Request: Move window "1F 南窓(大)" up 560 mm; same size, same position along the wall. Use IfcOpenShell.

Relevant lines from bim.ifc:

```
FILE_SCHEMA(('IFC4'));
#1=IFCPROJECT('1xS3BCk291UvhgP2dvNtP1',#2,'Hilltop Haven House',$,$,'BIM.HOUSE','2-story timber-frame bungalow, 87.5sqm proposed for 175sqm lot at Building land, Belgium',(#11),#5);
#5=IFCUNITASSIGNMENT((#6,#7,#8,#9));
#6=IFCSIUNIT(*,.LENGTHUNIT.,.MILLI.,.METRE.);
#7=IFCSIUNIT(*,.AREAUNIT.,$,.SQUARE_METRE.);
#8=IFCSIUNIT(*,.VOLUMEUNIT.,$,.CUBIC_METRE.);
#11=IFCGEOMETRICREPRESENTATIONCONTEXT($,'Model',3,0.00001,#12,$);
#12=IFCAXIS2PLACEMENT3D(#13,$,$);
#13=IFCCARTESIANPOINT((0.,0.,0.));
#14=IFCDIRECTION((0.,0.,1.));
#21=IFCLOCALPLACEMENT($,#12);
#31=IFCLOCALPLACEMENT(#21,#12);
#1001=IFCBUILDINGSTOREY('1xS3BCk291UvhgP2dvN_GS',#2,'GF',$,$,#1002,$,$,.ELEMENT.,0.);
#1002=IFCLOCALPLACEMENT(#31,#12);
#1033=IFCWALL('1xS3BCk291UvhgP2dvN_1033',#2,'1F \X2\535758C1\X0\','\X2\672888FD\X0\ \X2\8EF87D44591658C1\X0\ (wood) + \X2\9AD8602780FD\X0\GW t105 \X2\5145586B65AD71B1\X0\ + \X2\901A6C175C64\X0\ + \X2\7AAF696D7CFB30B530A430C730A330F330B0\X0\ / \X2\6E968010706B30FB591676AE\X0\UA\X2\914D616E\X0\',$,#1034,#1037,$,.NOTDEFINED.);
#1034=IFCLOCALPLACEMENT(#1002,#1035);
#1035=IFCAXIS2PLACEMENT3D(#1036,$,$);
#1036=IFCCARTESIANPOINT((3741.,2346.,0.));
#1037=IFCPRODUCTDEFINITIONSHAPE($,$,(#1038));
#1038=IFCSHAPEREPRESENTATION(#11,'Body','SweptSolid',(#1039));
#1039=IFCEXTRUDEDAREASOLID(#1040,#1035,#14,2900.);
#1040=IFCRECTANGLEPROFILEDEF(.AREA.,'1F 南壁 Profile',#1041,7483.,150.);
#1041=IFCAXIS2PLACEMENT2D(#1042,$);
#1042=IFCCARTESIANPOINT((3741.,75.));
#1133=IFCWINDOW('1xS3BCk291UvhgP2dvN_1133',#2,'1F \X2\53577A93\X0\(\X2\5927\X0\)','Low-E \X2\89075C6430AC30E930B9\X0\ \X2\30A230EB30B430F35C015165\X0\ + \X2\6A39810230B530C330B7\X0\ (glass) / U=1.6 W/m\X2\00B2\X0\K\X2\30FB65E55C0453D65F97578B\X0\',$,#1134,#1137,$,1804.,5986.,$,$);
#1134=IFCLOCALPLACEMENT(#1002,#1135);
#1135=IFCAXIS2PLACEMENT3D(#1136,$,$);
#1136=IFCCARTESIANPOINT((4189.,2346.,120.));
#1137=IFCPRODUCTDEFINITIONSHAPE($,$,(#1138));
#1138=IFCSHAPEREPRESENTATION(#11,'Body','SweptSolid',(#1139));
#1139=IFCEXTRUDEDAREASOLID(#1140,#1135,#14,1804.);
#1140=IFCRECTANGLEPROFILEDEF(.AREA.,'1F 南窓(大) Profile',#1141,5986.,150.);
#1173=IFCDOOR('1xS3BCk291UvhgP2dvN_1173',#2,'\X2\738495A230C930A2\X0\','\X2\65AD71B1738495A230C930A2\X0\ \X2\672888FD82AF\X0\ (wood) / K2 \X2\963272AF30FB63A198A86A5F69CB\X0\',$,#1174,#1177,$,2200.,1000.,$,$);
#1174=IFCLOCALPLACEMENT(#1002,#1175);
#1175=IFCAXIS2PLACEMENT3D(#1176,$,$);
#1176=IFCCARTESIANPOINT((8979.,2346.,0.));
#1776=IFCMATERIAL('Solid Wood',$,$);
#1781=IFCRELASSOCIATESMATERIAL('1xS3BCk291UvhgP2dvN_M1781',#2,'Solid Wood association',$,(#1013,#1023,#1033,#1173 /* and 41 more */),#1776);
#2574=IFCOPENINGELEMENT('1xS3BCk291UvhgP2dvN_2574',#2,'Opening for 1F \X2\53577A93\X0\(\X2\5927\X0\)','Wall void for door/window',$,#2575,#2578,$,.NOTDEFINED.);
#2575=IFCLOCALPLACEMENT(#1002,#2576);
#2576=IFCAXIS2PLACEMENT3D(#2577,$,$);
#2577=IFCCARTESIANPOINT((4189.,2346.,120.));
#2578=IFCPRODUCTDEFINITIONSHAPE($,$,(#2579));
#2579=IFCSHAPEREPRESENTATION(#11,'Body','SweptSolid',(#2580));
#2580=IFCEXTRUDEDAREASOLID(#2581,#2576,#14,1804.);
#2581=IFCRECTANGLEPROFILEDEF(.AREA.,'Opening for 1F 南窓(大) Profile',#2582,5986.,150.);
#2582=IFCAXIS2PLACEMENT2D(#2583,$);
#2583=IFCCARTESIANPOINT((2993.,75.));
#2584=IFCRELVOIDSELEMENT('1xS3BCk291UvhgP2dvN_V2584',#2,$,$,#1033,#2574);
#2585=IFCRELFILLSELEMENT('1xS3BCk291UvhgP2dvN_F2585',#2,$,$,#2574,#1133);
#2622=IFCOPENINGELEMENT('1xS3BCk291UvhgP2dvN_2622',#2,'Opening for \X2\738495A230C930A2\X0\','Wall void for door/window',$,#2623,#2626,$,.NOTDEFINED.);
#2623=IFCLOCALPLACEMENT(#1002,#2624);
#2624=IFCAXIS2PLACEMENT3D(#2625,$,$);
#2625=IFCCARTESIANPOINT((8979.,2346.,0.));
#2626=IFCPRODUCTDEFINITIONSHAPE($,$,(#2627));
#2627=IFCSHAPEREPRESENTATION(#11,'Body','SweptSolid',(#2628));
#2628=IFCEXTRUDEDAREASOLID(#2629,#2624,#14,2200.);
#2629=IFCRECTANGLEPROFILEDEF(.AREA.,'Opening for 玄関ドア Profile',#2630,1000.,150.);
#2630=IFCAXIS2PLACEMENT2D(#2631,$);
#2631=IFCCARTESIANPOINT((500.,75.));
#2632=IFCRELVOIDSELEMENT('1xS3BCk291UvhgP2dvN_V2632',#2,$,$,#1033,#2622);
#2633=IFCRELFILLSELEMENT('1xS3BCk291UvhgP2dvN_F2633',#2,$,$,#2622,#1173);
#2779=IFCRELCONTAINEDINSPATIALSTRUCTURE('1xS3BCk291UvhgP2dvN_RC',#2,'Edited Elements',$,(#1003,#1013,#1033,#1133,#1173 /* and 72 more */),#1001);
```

```python
import numpy as np
import ifcopenshell
import ifcopenshell.api.geometry
import ifcopenshell.util.placement
import ifcopenshell.util.unit

model = ifcopenshell.open("bim.ifc")
unit_scale = ifcopenshell.util.unit.calculate_unit_scale(model)

window = model.by_guid("1xS3BCk291UvhgP2dvN_1133")
opening = window.FillsVoids[0].RelatingOpeningElement
dz = 0.56 / unit_scale

shift = np.array([0.0, 0.0, dz])
# The window is not placed relative to its opening, so move both.
for product in (opening, window):
    matrix = ifcopenshell.util.placement.get_local_placement(product.ObjectPlacement)
    matrix[:3, 3] += shift
    ifcopenshell.api.geometry.edit_object_placement(model, product=product, matrix=matrix, is_si=False)

print(f"moved by {dz * unit_scale:+.3f} m")

model.write("bim-out.ifc")
```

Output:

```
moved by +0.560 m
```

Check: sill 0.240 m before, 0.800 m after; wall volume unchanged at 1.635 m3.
